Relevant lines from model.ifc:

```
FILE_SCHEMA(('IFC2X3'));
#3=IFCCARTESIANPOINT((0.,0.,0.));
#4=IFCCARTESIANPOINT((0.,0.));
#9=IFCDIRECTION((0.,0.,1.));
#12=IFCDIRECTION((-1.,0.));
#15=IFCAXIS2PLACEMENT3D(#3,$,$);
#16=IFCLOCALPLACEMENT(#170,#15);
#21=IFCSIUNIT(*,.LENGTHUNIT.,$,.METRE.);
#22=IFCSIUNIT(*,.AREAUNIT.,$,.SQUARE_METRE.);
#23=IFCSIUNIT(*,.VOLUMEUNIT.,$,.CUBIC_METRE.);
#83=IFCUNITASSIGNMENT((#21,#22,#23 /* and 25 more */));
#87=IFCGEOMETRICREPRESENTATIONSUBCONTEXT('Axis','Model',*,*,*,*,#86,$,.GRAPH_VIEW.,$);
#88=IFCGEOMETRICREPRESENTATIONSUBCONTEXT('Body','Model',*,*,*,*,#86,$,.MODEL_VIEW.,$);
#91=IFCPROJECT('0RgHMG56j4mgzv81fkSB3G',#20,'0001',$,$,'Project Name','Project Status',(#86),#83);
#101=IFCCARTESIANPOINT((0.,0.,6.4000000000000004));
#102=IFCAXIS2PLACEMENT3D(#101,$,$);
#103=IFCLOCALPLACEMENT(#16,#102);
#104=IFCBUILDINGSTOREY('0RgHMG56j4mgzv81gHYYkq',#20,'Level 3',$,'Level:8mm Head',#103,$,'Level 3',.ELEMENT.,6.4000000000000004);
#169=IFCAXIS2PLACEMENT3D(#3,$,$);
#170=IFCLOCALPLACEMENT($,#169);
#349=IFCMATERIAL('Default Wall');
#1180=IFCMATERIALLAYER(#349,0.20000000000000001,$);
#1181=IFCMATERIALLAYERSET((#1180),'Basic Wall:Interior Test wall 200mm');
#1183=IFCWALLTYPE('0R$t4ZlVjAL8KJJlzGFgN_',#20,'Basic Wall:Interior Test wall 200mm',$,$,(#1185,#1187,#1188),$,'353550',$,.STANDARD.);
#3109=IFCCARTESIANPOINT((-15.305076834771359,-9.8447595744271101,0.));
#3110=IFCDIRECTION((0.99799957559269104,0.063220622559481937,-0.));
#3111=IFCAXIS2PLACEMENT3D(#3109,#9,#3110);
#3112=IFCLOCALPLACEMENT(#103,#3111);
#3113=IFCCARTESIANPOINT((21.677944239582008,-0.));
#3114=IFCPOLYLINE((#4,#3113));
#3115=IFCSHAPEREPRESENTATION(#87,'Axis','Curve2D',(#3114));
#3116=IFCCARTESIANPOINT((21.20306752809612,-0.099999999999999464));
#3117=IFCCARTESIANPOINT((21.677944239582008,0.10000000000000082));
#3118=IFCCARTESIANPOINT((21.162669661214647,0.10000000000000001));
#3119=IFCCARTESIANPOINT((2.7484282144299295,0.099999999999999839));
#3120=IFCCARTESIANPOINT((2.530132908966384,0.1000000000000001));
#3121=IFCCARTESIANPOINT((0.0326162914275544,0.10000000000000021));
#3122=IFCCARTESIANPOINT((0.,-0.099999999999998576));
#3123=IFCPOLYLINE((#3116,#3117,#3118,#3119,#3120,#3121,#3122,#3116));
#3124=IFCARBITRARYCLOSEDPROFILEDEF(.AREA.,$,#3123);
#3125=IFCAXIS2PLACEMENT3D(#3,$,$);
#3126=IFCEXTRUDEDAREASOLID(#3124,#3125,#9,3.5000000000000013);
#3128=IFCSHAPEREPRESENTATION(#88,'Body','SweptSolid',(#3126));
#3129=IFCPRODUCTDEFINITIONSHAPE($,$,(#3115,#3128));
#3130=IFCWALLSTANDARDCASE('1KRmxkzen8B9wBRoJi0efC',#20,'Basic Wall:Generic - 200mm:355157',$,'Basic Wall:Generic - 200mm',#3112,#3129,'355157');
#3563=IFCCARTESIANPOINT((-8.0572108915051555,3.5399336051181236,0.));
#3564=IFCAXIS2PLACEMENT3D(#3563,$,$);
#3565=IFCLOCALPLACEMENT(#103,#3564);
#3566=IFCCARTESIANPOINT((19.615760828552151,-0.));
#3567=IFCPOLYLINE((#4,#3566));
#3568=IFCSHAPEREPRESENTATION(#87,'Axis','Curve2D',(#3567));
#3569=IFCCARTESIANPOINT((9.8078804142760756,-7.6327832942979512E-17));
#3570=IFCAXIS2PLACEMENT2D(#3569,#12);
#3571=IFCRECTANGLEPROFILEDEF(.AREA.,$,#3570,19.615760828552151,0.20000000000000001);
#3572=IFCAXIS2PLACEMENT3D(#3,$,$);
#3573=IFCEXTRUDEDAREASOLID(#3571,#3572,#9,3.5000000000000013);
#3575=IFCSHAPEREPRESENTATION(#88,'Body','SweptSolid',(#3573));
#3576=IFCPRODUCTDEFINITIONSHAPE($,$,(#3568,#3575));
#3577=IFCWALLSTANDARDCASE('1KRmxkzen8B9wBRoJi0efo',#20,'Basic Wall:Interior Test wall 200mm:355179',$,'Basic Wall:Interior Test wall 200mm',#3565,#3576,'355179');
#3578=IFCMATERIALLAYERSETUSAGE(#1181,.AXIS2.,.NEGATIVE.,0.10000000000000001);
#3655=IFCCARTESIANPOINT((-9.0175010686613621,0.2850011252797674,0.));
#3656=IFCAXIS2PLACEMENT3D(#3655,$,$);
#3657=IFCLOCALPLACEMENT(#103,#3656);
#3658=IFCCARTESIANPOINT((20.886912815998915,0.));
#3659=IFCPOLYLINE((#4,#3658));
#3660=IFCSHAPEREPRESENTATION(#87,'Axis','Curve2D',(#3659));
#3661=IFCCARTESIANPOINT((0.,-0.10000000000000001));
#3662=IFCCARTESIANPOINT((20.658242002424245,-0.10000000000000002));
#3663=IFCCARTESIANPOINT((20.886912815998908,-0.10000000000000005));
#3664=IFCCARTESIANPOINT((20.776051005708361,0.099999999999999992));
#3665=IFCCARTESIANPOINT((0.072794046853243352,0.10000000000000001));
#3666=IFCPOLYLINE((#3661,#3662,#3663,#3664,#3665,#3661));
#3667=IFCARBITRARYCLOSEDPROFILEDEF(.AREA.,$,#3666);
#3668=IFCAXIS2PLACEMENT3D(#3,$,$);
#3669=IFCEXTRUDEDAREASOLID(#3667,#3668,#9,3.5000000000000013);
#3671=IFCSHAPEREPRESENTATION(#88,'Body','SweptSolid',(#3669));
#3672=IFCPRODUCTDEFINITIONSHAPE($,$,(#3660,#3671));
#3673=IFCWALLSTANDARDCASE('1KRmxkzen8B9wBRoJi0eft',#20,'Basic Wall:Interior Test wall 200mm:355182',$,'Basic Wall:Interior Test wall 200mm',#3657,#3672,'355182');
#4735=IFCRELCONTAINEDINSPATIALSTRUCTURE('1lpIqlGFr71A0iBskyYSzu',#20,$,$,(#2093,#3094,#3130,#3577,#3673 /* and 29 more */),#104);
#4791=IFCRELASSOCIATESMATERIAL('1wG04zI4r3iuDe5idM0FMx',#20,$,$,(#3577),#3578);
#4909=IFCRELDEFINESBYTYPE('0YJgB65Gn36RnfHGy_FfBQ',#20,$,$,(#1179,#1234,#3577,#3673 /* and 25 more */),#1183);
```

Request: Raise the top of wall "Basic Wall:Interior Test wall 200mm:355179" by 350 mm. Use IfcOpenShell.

```python
import ifcopenshell
import ifcopenshell.geom
import ifcopenshell.util.representation
import ifcopenshell.util.shape
import ifcopenshell.util.unit

model = ifcopenshell.open("model.ifc")
unit_scale = ifcopenshell.util.unit.calculate_unit_scale(model)
settings = ifcopenshell.geom.settings()


def volume(element):
    """Net volume in cubic metres, openings subtracted."""
    shape = ifcopenshell.geom.create_shape(settings, element)
    return ifcopenshell.util.shape.get_volume(shape.geometry)


wall = model.by_id(3577)
before = volume(wall)

body = ifcopenshell.util.representation.get_representation(wall, "Model", "Body")
solid = body.Items[0]
old_height = solid.Depth
solid.Depth += 0.35 / unit_scale
after = volume(wall)

print(f"height {old_height:g} -> {solid.Depth:g}, volume {before:.3f} -> {after:.3f} m3")

model.write("model_edited.ifc")
```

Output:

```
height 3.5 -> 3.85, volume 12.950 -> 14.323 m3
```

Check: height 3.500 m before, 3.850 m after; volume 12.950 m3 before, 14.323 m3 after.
